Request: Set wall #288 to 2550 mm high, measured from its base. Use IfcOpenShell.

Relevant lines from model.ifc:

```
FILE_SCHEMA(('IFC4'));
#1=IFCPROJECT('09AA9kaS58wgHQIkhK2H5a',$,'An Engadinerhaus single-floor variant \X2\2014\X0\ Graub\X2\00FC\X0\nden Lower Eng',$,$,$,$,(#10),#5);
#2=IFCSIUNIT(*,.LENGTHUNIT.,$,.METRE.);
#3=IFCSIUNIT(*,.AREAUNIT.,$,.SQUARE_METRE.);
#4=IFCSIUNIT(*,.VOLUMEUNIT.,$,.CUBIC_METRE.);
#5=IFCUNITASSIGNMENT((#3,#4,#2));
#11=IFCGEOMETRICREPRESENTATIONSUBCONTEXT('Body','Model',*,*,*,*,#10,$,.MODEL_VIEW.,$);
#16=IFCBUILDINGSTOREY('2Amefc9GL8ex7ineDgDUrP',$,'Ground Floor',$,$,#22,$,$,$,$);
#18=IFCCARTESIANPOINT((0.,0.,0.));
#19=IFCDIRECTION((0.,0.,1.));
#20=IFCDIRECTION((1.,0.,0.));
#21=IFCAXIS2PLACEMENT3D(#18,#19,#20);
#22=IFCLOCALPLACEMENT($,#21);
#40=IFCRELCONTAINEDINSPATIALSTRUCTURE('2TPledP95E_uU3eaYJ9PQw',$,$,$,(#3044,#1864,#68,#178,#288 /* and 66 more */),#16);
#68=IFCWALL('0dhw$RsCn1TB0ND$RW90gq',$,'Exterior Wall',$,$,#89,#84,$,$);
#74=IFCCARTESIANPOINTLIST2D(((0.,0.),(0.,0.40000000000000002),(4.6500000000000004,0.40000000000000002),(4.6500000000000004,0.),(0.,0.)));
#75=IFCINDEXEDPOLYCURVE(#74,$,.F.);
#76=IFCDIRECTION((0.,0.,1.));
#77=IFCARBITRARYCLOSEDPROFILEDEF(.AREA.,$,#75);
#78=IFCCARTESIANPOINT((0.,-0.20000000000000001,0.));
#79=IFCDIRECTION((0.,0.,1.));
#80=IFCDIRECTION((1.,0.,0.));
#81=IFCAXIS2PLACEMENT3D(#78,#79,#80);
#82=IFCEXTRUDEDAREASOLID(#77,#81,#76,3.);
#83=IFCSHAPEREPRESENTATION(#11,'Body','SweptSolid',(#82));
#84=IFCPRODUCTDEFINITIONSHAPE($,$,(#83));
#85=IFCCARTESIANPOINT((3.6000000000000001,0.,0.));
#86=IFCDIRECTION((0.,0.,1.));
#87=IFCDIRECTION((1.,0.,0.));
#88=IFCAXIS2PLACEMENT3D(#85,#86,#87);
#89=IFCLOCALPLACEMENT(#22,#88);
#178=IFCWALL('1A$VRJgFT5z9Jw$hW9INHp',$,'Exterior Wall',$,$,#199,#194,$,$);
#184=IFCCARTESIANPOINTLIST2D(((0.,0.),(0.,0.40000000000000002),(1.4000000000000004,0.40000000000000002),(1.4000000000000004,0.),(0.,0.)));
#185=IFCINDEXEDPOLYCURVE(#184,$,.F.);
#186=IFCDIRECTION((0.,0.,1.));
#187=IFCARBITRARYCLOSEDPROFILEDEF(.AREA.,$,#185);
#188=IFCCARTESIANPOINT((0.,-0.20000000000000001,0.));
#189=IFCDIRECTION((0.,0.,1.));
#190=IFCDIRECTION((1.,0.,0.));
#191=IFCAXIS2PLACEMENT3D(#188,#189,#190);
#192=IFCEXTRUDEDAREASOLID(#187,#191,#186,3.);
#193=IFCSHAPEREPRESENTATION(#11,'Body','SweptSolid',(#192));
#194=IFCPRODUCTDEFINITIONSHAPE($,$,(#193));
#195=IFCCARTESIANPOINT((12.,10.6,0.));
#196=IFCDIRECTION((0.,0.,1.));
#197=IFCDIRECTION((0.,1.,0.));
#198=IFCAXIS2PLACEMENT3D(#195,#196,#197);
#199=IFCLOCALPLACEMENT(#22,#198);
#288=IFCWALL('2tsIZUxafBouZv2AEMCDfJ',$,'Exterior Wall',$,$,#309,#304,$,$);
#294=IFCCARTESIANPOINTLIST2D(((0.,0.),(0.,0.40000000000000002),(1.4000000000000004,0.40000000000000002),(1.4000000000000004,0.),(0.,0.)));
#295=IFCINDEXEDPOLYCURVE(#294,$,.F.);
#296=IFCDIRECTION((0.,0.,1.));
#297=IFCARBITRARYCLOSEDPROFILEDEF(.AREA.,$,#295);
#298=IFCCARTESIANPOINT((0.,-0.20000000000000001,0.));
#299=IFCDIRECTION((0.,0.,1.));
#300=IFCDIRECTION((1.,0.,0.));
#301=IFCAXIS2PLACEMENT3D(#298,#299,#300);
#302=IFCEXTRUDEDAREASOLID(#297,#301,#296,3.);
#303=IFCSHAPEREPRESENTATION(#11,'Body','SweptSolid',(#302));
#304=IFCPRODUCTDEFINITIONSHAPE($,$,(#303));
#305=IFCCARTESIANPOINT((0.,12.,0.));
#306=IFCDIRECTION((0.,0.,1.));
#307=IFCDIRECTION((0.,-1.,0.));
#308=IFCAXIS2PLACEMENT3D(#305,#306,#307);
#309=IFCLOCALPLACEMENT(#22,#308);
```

```python
import ifcopenshell
import ifcopenshell.geom
import ifcopenshell.util.representation
import ifcopenshell.util.shape
import ifcopenshell.util.unit

model = ifcopenshell.open("model.ifc")
unit_scale = ifcopenshell.util.unit.calculate_unit_scale(model)
settings = ifcopenshell.geom.settings()


def volume(element):
    """Net volume in cubic metres, openings subtracted."""
    shape = ifcopenshell.geom.create_shape(settings, element)
    return ifcopenshell.util.shape.get_volume(shape.geometry)


wall = model.by_id(288)
before = volume(wall)

body = ifcopenshell.util.representation.get_representation(wall, "Model", "Body")
solid = body.Items[0]
old_height = solid.Depth
solid.Depth = 2.55 / unit_scale
after = volume(wall)

print(f"height {old_height:g} -> {solid.Depth:g}, volume {before:.3f} -> {after:.3f} m3")

model.write("model_rev.ifc")
```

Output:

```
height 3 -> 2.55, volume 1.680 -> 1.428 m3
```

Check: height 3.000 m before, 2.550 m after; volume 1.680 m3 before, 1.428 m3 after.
